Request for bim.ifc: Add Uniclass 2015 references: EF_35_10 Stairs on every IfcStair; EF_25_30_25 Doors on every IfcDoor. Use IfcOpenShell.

First a look at what the model holds.

```python
import ifcopenshell

model = ifcopenshell.open("bim.ifc")
print(model.schema)
print("classifications:", [c.Name for c in model.by_type("IfcClassification")])
for ifc_class in ("IfcDoor", "IfcRoof", "IfcStair", "IfcWall", "IfcWindow"):
    print(ifc_class, len(model.by_type(ifc_class)))
```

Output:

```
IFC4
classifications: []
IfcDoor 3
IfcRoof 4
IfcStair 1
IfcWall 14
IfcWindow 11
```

```python
import ifcopenshell
import ifcopenshell.api.classification

model = ifcopenshell.open("bim.ifc")

system = ifcopenshell.api.classification.add_classification(model, classification="Uniclass 2015")

codes = {
    "IfcStair": ("EF_35_10", "Stairs"),
    "IfcDoor": ("EF_25_30_25", "Doors"),
}
for ifc_class, (code, name) in codes.items():
    products = model.by_type(ifc_class)
    ifcopenshell.api.classification.add_reference(
        model, products=products, classification=system, identification=code, name=name
    )
    print(code, len(products))

model.write("bim_v2.ifc")
```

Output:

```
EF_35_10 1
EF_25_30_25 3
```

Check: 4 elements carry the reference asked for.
